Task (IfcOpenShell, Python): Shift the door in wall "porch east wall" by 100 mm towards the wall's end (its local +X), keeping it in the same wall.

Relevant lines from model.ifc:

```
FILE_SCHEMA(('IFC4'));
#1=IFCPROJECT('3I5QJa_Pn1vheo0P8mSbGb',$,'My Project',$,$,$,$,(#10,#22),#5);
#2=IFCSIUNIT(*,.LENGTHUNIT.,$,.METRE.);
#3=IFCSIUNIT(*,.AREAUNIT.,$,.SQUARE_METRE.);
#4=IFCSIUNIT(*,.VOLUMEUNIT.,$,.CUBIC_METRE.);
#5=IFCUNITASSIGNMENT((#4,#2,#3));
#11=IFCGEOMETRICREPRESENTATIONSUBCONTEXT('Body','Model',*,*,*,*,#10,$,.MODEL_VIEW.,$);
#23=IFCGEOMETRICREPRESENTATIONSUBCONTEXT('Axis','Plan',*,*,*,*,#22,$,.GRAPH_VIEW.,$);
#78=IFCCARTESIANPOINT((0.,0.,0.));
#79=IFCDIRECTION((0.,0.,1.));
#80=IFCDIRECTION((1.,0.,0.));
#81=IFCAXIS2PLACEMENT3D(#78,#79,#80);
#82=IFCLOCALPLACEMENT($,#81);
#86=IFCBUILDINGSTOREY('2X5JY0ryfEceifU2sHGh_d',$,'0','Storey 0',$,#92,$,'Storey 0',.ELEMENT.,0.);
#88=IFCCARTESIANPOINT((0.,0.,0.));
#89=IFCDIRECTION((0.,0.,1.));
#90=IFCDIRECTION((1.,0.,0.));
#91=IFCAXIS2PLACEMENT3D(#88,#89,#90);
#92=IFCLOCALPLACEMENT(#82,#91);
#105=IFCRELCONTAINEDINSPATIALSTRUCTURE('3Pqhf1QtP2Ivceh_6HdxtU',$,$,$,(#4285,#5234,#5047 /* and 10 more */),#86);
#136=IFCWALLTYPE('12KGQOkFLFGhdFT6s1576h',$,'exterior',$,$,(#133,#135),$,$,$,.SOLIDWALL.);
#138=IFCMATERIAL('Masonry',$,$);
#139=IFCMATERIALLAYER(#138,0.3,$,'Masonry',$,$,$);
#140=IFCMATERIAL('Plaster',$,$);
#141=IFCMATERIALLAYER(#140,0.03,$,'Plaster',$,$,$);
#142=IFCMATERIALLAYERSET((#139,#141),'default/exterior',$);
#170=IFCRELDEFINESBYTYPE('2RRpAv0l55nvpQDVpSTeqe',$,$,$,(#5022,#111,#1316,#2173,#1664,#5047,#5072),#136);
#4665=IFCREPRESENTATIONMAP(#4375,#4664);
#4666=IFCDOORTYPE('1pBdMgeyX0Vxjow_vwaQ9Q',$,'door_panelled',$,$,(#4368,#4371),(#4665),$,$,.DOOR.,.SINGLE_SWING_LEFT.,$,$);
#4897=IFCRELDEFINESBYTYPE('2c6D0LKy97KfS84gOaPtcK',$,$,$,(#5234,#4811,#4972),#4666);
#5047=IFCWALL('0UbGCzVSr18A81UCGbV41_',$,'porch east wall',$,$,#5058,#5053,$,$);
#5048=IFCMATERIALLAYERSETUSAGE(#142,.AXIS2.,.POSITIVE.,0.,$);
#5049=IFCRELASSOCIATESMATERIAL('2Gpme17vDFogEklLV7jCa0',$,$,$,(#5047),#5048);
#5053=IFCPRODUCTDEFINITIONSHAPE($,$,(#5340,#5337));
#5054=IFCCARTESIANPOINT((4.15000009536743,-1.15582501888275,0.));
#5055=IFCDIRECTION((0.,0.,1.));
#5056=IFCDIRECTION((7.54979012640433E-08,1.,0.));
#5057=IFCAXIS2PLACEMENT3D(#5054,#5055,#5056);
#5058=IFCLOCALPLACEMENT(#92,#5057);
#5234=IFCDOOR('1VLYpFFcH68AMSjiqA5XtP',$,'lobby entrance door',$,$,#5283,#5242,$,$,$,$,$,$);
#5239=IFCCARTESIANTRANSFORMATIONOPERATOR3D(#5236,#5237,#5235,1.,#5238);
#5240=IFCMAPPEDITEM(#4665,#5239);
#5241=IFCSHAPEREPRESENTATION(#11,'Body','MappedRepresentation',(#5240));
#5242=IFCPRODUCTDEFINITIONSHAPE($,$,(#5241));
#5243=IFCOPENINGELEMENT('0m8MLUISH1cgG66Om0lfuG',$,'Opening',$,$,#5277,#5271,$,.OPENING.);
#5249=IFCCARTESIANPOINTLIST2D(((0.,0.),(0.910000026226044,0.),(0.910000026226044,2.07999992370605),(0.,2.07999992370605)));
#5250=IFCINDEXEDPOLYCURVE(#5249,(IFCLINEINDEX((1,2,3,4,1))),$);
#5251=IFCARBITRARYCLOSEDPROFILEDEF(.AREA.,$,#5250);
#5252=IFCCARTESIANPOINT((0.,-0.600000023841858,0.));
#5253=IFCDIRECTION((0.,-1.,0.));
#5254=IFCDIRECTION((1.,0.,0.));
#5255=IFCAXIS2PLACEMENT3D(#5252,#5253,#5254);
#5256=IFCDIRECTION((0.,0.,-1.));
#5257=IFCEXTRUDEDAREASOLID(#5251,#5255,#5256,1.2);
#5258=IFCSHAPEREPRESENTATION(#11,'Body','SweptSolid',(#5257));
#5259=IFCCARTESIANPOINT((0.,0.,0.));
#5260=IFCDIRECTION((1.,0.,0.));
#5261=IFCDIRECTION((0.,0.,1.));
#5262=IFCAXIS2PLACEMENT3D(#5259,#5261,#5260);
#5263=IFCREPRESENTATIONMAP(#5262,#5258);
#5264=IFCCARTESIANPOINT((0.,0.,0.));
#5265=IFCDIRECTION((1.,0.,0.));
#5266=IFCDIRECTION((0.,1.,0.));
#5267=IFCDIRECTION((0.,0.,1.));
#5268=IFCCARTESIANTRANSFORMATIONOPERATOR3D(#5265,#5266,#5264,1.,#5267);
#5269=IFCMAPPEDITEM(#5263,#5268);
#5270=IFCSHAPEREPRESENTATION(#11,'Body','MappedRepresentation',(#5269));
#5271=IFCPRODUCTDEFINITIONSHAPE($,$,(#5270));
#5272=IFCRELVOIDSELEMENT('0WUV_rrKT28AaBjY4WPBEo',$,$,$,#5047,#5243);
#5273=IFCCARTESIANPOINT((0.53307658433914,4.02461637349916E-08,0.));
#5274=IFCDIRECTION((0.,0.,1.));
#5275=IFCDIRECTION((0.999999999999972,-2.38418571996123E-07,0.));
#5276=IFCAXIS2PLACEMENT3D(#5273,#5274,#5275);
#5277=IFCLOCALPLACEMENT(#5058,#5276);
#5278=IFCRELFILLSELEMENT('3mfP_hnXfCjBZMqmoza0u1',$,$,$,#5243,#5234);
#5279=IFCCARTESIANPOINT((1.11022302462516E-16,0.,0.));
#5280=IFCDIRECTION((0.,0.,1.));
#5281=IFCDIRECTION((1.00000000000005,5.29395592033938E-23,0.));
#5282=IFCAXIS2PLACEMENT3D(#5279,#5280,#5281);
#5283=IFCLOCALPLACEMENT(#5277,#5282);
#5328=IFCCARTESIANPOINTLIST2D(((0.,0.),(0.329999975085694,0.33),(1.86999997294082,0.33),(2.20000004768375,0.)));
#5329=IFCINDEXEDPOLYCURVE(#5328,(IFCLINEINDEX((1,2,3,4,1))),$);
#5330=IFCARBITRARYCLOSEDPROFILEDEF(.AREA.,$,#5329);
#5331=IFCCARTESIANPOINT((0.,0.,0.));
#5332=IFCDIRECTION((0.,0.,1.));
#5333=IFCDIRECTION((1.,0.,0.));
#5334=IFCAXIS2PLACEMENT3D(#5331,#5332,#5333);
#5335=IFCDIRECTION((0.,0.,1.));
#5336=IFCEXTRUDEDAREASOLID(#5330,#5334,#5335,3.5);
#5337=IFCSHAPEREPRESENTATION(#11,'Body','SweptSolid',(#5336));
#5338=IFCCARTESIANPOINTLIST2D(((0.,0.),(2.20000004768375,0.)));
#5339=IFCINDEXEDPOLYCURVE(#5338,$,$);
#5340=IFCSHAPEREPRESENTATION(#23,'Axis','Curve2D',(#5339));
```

```python
import ifcopenshell
import ifcopenshell.api.geometry
import ifcopenshell.util.placement
import ifcopenshell.util.unit

model = ifcopenshell.open("model.ifc")
unit_scale = ifcopenshell.util.unit.calculate_unit_scale(model)

door = model.by_guid("1VLYpFFcH68AMSjiqA5XtP")
opening = door.FillsVoids[0].RelatingOpeningElement
wall = opening.VoidsElements[0].RelatingBuildingElement

wall_matrix = ifcopenshell.util.placement.get_local_placement(wall.ObjectPlacement)
shift = wall_matrix[:3, 0] * 0.1 / unit_scale
before = ifcopenshell.util.placement.get_local_placement(door.ObjectPlacement)[:3, 3].copy()

# The door is placed relative to its opening, so it follows when the opening moves.
matrix = ifcopenshell.util.placement.get_local_placement(opening.ObjectPlacement)
matrix[:3, 3] += shift
ifcopenshell.api.geometry.edit_object_placement(
    model, product=opening, matrix=matrix, is_si=False, should_transform_children=True
)

after = ifcopenshell.util.placement.get_local_placement(door.ObjectPlacement)[:3, 3]
print("door moved by", (after - before).round(3) + 0.0)

model.write("model-out.ifc")
```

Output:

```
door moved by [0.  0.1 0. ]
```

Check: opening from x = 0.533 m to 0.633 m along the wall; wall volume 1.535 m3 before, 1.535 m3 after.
